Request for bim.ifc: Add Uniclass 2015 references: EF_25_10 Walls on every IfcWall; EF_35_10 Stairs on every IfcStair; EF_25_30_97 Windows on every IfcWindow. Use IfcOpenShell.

First a look at what the model holds.

```python
import ifcopenshell

model = ifcopenshell.open("bim.ifc")
print(model.schema)
print("classifications:", [c.Name for c in model.by_type("IfcClassification")])
for ifc_class in ("IfcDoor", "IfcRoof", "IfcStair", "IfcWall", "IfcWindow"):
    print(ifc_class, len(model.by_type(ifc_class)))
```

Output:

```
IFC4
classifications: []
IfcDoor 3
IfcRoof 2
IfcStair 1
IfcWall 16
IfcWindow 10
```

```python
import ifcopenshell
import ifcopenshell.api.classification

model = ifcopenshell.open("bim.ifc")

system = ifcopenshell.api.classification.add_classification(model, classification="Uniclass 2015")

codes = {
    "IfcWall": ("EF_25_10", "Walls"),
    "IfcStair": ("EF_35_10", "Stairs"),
    "IfcWindow": ("EF_25_30_97", "Windows"),
}
for ifc_class, (code, name) in codes.items():
    products = model.by_type(ifc_class)
    ifcopenshell.api.classification.add_reference(
        model, products=products, classification=system, identification=code, name=name
    )
    print(code, len(products))

model.write("bim_edited.ifc")
```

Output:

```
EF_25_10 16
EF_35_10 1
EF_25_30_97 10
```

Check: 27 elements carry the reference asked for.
